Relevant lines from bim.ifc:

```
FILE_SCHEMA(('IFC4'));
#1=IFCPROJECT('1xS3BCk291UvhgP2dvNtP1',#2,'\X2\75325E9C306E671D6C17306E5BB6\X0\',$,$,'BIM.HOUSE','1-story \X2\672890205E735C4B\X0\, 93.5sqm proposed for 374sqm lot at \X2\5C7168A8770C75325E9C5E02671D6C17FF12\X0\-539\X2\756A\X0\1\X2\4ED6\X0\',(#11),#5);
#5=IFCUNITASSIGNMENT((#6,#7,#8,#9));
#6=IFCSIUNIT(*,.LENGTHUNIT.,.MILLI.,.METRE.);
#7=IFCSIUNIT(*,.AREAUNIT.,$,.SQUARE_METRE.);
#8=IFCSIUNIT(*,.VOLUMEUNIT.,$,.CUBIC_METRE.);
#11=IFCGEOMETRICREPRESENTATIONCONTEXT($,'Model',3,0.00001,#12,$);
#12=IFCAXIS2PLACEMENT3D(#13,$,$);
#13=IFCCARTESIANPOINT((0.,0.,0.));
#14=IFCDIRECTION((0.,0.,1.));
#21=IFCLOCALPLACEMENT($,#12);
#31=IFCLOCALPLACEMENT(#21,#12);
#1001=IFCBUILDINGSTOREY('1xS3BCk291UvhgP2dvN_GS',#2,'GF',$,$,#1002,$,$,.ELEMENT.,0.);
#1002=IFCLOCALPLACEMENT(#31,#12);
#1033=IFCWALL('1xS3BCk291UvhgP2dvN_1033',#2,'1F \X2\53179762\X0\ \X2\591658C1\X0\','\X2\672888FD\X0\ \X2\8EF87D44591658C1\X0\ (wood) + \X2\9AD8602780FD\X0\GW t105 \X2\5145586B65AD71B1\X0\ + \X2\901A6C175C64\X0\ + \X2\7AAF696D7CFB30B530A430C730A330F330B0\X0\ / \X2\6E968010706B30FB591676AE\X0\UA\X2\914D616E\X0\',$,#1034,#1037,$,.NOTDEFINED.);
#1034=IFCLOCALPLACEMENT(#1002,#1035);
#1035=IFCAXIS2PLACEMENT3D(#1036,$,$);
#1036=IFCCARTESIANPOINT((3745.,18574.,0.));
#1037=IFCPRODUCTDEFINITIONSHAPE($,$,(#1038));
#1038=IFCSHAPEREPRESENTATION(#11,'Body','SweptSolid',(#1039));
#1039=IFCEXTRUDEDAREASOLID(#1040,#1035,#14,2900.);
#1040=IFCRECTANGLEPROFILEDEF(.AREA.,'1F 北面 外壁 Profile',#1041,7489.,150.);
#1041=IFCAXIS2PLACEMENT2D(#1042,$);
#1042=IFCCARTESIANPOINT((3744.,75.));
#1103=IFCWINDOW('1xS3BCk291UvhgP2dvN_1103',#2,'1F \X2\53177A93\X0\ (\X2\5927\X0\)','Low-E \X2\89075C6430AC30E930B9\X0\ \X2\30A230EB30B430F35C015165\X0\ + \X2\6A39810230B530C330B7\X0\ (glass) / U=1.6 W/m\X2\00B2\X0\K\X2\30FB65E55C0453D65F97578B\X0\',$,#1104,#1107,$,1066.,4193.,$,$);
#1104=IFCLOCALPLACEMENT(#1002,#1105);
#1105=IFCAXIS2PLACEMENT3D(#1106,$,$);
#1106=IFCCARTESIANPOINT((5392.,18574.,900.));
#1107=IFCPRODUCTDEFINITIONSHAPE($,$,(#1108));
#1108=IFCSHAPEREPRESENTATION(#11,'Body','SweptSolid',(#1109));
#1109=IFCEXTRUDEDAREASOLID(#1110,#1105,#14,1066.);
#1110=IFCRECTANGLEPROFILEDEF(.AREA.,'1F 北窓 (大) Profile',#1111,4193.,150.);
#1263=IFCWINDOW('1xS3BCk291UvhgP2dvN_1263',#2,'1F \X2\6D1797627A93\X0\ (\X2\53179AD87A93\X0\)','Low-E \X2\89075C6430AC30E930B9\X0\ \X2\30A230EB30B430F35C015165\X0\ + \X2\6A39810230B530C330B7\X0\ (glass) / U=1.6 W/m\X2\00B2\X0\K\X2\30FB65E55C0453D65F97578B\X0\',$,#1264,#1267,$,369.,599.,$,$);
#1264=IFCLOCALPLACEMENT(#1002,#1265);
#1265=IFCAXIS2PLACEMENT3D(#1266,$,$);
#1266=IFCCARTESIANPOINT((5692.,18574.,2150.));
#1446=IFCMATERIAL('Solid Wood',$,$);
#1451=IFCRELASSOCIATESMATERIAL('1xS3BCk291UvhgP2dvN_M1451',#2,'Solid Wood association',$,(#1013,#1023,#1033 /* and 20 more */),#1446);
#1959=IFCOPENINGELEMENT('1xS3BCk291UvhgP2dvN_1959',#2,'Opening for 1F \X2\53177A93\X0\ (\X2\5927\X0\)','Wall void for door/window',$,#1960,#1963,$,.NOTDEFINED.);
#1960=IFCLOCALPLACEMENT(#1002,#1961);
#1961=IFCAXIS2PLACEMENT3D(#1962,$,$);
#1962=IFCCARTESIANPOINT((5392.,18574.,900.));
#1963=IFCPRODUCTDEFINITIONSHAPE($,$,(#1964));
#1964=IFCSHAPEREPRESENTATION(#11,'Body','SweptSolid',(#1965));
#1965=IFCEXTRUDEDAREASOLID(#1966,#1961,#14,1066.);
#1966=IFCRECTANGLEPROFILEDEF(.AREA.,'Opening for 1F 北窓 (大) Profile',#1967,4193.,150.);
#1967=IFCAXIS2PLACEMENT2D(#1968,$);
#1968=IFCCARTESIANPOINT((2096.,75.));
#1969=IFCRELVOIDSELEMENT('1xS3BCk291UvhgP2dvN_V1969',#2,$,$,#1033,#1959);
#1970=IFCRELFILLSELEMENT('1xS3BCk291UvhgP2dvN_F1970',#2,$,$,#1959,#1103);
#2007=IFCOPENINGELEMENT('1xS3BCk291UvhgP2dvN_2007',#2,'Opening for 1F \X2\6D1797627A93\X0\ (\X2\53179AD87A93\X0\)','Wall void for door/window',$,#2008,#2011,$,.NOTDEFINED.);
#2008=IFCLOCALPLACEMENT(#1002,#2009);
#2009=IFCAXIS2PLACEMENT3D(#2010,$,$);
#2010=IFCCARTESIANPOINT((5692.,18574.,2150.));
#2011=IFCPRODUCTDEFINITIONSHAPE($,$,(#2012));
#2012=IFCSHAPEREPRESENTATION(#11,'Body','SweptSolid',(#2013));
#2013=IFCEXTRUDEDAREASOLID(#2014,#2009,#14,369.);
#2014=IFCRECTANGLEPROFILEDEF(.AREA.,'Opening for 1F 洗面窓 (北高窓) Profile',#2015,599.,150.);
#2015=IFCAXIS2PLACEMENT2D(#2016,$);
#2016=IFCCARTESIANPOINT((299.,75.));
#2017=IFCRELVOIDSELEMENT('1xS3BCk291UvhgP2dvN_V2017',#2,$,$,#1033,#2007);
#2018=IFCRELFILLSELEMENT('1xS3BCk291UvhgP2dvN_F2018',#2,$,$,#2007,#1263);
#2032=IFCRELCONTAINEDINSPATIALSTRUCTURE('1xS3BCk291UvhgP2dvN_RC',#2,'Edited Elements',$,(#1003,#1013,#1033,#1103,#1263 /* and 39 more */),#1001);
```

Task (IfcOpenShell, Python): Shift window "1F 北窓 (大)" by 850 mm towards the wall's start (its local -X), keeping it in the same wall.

```python
import ifcopenshell
import ifcopenshell.api.geometry
import ifcopenshell.util.placement
import ifcopenshell.util.unit

model = ifcopenshell.open("bim.ifc")
unit_scale = ifcopenshell.util.unit.calculate_unit_scale(model)

window = model.by_id(1103)
opening = window.FillsVoids[0].RelatingOpeningElement
wall = opening.VoidsElements[0].RelatingBuildingElement

wall_matrix = ifcopenshell.util.placement.get_local_placement(wall.ObjectPlacement)
shift = wall_matrix[:3, 0] * -0.85 / unit_scale
before = ifcopenshell.util.placement.get_local_placement(window.ObjectPlacement)[:3, 3].copy()

# The window is not placed relative to its opening, so move both.
for product in (opening, window):
    matrix = ifcopenshell.util.placement.get_local_placement(product.ObjectPlacement)
    matrix[:3, 3] += shift
    ifcopenshell.api.geometry.edit_object_placement(model, product=product, matrix=matrix, is_si=False)

after = ifcopenshell.util.placement.get_local_placement(window.ObjectPlacement)[:3, 3]
print("window moved by", (after - before).round(3) + 0.0)

model.write("bim-out.ifc")
```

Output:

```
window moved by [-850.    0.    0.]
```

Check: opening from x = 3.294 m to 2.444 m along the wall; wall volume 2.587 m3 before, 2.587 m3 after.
